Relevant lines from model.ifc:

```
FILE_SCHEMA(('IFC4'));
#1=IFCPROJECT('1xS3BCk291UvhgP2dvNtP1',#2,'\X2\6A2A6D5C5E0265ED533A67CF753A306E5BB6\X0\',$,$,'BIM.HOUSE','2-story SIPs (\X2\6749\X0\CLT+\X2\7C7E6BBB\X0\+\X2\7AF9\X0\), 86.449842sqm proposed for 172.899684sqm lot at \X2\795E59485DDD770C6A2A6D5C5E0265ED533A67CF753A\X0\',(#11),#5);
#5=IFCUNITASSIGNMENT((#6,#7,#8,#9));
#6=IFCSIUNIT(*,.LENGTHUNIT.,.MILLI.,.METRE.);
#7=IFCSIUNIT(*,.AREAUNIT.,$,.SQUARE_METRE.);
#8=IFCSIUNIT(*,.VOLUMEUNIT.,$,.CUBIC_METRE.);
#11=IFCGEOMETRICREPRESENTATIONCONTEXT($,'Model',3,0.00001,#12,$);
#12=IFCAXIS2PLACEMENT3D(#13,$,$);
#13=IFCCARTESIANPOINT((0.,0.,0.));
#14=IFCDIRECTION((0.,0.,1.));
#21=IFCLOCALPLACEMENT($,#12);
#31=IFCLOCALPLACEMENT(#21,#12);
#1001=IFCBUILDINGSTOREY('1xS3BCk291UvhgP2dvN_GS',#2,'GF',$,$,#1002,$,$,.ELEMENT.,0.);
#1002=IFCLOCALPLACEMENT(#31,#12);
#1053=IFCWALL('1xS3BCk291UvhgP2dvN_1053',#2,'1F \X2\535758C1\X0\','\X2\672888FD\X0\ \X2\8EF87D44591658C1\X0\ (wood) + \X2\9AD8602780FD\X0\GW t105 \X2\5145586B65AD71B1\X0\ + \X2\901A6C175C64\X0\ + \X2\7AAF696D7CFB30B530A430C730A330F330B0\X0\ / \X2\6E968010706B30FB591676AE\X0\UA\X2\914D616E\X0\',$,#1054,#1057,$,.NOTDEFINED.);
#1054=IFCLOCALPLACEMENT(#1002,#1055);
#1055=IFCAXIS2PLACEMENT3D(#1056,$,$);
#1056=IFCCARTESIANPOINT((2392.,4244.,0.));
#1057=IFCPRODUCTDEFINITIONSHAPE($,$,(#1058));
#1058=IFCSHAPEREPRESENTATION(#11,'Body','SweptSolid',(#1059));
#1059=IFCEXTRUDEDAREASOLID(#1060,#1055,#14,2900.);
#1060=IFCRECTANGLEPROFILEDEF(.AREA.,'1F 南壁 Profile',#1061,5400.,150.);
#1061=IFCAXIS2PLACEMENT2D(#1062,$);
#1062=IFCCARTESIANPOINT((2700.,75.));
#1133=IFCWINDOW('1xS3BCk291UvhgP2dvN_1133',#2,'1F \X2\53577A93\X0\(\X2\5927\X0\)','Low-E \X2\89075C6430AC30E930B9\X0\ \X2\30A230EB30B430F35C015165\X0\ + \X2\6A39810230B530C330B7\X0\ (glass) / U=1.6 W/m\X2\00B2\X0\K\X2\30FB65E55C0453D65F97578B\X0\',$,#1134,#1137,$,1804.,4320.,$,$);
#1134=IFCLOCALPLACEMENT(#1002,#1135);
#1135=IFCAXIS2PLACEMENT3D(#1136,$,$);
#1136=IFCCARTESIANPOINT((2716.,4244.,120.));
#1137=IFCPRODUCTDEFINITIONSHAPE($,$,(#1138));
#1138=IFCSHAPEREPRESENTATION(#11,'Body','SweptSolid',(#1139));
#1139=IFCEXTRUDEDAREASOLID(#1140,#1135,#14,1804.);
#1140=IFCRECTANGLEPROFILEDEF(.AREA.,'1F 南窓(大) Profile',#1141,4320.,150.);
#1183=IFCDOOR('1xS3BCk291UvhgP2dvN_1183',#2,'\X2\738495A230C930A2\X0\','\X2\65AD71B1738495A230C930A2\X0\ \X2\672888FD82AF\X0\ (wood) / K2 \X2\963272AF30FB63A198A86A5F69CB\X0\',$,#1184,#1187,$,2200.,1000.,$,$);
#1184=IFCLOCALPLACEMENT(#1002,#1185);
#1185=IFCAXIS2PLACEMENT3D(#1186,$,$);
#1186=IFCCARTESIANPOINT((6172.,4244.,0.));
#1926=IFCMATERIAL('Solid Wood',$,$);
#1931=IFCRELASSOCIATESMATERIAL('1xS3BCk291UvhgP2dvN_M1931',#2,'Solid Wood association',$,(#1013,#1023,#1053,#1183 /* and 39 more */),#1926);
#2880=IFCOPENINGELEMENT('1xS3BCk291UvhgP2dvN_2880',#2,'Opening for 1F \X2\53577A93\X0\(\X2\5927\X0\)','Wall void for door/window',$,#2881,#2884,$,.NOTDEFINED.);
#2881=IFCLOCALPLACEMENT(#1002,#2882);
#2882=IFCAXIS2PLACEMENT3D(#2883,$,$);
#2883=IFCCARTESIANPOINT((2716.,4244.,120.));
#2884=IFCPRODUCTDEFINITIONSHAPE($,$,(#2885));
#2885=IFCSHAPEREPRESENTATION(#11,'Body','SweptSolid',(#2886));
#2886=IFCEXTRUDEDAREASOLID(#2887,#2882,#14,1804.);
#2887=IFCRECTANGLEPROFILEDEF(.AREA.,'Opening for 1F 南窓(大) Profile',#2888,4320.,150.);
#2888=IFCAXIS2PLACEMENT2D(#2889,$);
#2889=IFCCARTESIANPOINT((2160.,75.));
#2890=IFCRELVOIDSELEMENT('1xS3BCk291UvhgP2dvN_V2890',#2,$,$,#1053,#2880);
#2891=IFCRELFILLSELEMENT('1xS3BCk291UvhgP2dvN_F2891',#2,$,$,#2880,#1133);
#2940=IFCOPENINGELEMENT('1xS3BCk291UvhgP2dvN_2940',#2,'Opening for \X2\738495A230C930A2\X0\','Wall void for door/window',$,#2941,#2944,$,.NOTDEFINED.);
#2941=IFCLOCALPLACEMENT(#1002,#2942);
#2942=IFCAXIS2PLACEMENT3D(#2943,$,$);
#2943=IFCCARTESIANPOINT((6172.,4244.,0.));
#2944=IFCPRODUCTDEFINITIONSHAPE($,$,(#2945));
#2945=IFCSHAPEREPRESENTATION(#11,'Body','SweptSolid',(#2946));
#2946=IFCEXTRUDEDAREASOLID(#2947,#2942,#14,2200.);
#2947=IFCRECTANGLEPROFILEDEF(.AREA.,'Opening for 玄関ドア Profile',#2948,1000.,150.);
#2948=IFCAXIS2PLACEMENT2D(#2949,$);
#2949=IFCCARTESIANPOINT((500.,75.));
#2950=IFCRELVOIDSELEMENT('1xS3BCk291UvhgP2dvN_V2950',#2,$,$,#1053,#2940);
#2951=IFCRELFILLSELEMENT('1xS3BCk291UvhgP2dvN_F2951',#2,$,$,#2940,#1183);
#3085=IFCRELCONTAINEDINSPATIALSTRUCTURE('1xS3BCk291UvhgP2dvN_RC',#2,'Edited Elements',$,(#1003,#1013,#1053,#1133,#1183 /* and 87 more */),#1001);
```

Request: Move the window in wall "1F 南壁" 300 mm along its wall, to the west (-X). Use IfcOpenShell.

```python
import ifcopenshell
import ifcopenshell.api.geometry
import ifcopenshell.util.placement
import ifcopenshell.util.unit

model = ifcopenshell.open("model.ifc")
unit_scale = ifcopenshell.util.unit.calculate_unit_scale(model)

window = model.by_guid("1xS3BCk291UvhgP2dvN_1133")
opening = window.FillsVoids[0].RelatingOpeningElement
wall = opening.VoidsElements[0].RelatingBuildingElement

wall_matrix = ifcopenshell.util.placement.get_local_placement(wall.ObjectPlacement)
shift = wall_matrix[:3, 0] * -0.3 / unit_scale
before = ifcopenshell.util.placement.get_local_placement(window.ObjectPlacement)[:3, 3].copy()

# The window is not placed relative to its opening, so move both.
for product in (opening, window):
    matrix = ifcopenshell.util.placement.get_local_placement(product.ObjectPlacement)
    matrix[:3, 3] += shift
    ifcopenshell.api.geometry.edit_object_placement(model, product=product, matrix=matrix, is_si=False)

after = ifcopenshell.util.placement.get_local_placement(window.ObjectPlacement)[:3, 3]
print("window moved by", (after - before).round(3) + 0.0)

model.write("model-out.ifc")
```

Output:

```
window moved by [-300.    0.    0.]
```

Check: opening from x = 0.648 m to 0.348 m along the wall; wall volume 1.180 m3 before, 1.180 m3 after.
